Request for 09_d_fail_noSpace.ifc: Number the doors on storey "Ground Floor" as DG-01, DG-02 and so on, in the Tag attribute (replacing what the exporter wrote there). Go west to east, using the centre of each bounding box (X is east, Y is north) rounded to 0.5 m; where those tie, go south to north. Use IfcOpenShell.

First a look at what the model holds.

```python
import ifcopenshell
import ifcopenshell.util.element
import ifcopenshell.util.placement

model = ifcopenshell.open("09_d_fail_noSpace.ifc")
print(model.schema)
storey = next(s for s in model.by_type("IfcBuildingStorey") if s.Name == "Ground Floor")
doors = [e for e in ifcopenshell.util.element.get_decomposition(storey) if e.is_a("IfcDoor")]
for e in sorted(doors, key=lambda e: e.id()):
    origin = ifcopenshell.util.placement.get_local_placement(e.ObjectPlacement)[:3, 3]
    print(e.id(), e.Tag, e.Name, origin.round(2) + 0.0, sep=" | ")
```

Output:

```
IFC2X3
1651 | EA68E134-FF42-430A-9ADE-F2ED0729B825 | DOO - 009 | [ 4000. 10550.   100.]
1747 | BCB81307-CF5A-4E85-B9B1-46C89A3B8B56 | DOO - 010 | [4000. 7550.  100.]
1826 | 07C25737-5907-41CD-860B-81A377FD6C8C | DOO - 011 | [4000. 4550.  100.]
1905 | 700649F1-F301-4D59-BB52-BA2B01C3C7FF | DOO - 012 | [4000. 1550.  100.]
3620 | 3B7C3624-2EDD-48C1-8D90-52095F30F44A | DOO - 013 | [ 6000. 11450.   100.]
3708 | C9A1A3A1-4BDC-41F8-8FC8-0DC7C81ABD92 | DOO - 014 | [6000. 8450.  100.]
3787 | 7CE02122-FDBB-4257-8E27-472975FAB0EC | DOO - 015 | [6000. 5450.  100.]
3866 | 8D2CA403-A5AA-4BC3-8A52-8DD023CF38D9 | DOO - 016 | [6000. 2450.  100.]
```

```python
import ifcopenshell
import ifcopenshell.geom
import ifcopenshell.util.element
import ifcopenshell.util.shape

model = ifcopenshell.open("09_d_fail_noSpace.ifc")
settings = ifcopenshell.geom.settings()
settings.set("use-world-coords", True)


def centre(element):
    shape = ifcopenshell.geom.create_shape(settings, element)
    return ifcopenshell.util.shape.get_bbox_centroid(shape.geometry)


storey = next(s for s in model.by_type("IfcBuildingStorey") if s.Name == "Ground Floor")
doors = [e for e in ifcopenshell.util.element.get_decomposition(storey) if e.is_a("IfcDoor")]

# Insertion points can sit at a corner or the storey origin, so sort by the geometry (in metres).
centres = {e: centre(e) for e in doors}
doors.sort(key=lambda e: (round(centres[e][0] / 0.5), centres[e][1]))

for i, e in enumerate(doors, start=1):
    number = f"DG-{i:02d}"
    e.Tag = number
    print(e.id(), number)

model.write("09_d_fail_noSpace_edited.ifc")
```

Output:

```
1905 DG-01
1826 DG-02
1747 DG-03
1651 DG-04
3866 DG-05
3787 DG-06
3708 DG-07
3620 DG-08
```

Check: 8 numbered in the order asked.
